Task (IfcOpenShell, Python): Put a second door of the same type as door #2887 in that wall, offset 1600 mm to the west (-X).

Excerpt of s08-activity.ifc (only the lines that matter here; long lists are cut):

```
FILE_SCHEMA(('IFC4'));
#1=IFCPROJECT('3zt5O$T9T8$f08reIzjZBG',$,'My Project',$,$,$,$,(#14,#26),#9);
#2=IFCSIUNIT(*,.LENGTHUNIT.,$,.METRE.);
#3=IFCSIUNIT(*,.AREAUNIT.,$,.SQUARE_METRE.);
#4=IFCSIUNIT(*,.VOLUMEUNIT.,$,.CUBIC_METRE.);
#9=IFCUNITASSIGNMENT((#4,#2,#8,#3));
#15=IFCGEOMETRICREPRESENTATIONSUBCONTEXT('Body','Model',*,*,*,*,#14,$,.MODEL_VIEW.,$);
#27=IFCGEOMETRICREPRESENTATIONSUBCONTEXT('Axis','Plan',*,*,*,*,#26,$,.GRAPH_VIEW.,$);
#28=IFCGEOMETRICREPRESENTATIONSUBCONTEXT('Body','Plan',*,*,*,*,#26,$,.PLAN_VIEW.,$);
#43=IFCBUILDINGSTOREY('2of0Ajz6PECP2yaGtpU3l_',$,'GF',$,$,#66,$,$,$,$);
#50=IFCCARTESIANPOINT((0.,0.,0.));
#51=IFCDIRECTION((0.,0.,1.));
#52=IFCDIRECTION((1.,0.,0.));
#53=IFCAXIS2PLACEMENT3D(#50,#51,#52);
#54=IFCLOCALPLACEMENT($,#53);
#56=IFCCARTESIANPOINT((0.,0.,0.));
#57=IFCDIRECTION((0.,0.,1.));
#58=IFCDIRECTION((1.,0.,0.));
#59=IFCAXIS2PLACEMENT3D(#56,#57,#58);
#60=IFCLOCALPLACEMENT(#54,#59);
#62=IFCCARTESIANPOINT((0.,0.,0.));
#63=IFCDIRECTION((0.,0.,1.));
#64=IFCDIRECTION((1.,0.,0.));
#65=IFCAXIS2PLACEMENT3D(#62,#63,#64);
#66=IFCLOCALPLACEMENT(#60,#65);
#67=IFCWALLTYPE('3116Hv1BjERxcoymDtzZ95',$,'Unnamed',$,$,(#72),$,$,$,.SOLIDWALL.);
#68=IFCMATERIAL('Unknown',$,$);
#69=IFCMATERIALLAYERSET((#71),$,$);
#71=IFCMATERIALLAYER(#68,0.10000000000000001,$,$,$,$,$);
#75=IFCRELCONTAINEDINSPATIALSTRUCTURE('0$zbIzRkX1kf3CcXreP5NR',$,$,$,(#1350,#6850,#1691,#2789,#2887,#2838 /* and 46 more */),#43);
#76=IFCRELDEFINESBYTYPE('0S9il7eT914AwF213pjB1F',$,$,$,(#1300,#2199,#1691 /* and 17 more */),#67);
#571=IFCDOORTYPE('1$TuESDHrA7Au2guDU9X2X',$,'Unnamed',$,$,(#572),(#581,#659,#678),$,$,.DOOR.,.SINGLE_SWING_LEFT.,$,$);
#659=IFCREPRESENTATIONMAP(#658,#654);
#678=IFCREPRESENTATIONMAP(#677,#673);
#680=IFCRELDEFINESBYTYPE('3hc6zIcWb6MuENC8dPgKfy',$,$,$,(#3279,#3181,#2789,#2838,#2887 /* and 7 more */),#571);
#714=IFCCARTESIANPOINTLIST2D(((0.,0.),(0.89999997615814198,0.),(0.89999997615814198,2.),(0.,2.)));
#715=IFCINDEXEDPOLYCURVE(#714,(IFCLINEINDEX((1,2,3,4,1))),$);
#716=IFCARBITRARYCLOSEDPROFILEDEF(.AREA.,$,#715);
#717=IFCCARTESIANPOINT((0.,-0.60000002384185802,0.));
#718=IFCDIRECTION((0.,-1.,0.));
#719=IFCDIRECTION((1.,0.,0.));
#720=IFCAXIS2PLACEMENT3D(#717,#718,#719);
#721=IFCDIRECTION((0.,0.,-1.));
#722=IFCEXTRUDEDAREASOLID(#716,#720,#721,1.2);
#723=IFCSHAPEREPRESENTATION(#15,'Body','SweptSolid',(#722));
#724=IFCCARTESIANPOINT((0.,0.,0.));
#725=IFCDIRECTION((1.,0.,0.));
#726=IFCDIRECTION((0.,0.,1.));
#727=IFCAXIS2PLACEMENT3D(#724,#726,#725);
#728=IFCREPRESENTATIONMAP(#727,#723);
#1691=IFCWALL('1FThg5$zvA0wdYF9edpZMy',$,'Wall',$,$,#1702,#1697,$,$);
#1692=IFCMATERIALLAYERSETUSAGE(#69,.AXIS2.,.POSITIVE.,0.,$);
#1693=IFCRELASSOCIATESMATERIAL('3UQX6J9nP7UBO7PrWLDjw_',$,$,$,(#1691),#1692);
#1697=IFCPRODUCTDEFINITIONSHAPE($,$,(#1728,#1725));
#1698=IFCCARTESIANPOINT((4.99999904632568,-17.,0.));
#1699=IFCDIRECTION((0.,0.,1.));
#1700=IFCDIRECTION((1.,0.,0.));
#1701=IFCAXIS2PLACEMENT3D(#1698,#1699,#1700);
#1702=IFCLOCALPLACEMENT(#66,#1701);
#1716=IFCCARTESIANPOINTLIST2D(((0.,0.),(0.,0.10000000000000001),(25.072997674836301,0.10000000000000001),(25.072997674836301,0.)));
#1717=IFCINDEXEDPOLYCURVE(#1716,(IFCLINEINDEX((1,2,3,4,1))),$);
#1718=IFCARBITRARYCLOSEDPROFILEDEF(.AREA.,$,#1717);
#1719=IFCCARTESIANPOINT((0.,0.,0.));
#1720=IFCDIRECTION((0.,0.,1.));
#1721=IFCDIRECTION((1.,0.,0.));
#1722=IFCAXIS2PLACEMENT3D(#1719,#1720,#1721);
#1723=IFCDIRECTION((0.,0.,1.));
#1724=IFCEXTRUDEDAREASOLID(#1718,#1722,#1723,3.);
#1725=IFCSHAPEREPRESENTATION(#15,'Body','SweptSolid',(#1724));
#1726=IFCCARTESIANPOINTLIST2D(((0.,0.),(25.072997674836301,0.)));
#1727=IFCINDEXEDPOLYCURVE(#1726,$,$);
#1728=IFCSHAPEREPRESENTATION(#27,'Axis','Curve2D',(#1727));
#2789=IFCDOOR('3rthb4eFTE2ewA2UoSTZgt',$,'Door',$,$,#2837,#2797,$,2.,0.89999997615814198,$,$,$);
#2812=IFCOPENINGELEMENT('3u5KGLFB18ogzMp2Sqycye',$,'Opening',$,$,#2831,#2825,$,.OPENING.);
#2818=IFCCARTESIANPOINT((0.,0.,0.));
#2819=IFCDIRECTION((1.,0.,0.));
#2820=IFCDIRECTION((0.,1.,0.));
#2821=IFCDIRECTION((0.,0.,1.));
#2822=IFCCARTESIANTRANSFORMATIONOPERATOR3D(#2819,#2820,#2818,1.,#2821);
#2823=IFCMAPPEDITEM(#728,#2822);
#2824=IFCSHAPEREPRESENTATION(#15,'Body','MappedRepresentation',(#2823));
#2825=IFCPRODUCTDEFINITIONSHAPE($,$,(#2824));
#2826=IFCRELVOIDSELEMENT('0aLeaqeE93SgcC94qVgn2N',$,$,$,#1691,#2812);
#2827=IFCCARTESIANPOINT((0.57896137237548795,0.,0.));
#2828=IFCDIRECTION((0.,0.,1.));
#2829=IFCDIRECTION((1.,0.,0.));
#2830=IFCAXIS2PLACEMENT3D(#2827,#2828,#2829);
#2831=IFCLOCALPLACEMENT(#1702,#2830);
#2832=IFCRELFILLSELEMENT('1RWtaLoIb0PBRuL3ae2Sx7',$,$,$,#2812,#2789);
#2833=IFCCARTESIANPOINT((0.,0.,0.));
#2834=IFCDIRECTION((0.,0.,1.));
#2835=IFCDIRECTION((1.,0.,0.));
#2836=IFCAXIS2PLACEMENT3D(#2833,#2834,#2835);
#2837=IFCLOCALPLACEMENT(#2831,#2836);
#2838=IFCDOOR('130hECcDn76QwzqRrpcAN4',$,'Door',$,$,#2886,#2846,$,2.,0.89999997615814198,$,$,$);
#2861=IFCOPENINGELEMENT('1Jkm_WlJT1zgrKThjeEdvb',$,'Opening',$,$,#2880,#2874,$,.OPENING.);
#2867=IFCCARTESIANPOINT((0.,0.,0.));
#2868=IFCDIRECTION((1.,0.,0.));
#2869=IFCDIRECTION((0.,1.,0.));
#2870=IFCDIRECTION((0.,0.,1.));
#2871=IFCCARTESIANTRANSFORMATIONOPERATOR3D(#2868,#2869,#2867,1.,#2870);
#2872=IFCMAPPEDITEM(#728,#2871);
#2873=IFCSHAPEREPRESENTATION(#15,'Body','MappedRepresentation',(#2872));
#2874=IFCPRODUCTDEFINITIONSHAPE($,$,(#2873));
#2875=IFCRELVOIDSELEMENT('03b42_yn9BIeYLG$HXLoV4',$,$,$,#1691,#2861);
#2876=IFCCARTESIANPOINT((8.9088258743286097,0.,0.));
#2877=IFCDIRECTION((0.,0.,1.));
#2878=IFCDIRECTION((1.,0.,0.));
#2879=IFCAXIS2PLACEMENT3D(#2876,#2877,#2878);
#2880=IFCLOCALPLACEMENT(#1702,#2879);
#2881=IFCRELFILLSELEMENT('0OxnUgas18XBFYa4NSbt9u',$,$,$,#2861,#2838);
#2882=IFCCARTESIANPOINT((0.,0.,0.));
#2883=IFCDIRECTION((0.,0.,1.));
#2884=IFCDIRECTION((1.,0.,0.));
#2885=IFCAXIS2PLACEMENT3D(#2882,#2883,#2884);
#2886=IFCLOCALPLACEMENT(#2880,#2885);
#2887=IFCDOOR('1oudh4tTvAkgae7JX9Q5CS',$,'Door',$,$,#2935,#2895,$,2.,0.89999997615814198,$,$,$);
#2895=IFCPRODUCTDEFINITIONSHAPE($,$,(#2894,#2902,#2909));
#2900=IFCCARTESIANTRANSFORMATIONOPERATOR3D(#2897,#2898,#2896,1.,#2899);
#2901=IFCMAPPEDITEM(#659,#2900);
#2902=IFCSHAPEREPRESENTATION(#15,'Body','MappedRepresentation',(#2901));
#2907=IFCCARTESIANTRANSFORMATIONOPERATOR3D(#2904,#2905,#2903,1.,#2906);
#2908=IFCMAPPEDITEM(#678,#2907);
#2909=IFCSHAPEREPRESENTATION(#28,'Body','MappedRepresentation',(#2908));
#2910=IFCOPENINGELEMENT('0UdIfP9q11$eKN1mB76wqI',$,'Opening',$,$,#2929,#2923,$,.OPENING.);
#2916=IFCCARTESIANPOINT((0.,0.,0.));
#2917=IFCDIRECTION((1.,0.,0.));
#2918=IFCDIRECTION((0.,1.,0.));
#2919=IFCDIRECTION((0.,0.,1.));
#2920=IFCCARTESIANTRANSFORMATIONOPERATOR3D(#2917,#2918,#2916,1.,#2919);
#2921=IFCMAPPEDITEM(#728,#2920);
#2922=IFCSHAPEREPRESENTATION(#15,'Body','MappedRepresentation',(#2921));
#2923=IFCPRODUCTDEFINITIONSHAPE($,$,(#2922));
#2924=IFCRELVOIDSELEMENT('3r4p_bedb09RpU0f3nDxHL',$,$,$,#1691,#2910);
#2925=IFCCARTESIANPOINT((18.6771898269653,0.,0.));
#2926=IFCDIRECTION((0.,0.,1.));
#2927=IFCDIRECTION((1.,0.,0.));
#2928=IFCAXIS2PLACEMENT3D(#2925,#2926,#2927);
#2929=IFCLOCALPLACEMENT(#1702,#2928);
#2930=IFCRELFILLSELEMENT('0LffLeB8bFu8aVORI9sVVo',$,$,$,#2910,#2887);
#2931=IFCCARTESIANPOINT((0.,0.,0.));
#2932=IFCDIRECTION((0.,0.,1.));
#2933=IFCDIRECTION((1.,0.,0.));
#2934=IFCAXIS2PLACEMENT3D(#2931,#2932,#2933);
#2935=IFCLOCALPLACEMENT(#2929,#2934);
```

```python
import ifcopenshell
import ifcopenshell.api.feature
import ifcopenshell.api.geometry
import ifcopenshell.api.root
import ifcopenshell.geom
import ifcopenshell.util.element
import ifcopenshell.util.placement
import ifcopenshell.util.shape

model = ifcopenshell.open("s08-activity.ifc")
settings = ifcopenshell.geom.settings()


def volume(element):
    """Net volume in cubic metres, openings subtracted."""
    shape = ifcopenshell.geom.create_shape(settings, element)
    return ifcopenshell.util.shape.get_volume(shape.geometry)


door = model.by_guid("1oudh4tTvAkgae7JX9Q5CS")
opening = door.FillsVoids[0].RelatingOpeningElement
wall = opening.VoidsElements[0].RelatingBuildingElement
before = volume(wall)
shift = ifcopenshell.util.placement.get_local_placement(wall.ObjectPlacement)[:3, 0] * -1.6

# copy_class copies the void relationship, type, container and properties, but no geometry.
new_opening = ifcopenshell.api.root.copy_class(model, product=opening)
new_opening.Representation = ifcopenshell.util.element.copy_deep(
    model, opening.Representation, exclude=["IfcGeometricRepresentationContext", "IfcRepresentationMap"]
)
new_door = ifcopenshell.api.root.copy_class(model, product=door)
new_door.Representation = ifcopenshell.util.element.copy_deep(
    model, door.Representation, exclude=["IfcGeometricRepresentationContext", "IfcRepresentationMap"]
)
ifcopenshell.api.feature.add_filling(model, opening=new_opening, element=new_door)

for old, new in ((opening, new_opening), (door, new_door)):
    matrix = ifcopenshell.util.placement.get_local_placement(old.ObjectPlacement)
    matrix[:3, 3] += shift
    ifcopenshell.api.geometry.edit_object_placement(model, product=new, matrix=matrix, is_si=False)

after = volume(wall)

print(f"wall volume {before:.3f} -> {after:.3f} m3")

model.write("s08-activity_rev.ifc")
```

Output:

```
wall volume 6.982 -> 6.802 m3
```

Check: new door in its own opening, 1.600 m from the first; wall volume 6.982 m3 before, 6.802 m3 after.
